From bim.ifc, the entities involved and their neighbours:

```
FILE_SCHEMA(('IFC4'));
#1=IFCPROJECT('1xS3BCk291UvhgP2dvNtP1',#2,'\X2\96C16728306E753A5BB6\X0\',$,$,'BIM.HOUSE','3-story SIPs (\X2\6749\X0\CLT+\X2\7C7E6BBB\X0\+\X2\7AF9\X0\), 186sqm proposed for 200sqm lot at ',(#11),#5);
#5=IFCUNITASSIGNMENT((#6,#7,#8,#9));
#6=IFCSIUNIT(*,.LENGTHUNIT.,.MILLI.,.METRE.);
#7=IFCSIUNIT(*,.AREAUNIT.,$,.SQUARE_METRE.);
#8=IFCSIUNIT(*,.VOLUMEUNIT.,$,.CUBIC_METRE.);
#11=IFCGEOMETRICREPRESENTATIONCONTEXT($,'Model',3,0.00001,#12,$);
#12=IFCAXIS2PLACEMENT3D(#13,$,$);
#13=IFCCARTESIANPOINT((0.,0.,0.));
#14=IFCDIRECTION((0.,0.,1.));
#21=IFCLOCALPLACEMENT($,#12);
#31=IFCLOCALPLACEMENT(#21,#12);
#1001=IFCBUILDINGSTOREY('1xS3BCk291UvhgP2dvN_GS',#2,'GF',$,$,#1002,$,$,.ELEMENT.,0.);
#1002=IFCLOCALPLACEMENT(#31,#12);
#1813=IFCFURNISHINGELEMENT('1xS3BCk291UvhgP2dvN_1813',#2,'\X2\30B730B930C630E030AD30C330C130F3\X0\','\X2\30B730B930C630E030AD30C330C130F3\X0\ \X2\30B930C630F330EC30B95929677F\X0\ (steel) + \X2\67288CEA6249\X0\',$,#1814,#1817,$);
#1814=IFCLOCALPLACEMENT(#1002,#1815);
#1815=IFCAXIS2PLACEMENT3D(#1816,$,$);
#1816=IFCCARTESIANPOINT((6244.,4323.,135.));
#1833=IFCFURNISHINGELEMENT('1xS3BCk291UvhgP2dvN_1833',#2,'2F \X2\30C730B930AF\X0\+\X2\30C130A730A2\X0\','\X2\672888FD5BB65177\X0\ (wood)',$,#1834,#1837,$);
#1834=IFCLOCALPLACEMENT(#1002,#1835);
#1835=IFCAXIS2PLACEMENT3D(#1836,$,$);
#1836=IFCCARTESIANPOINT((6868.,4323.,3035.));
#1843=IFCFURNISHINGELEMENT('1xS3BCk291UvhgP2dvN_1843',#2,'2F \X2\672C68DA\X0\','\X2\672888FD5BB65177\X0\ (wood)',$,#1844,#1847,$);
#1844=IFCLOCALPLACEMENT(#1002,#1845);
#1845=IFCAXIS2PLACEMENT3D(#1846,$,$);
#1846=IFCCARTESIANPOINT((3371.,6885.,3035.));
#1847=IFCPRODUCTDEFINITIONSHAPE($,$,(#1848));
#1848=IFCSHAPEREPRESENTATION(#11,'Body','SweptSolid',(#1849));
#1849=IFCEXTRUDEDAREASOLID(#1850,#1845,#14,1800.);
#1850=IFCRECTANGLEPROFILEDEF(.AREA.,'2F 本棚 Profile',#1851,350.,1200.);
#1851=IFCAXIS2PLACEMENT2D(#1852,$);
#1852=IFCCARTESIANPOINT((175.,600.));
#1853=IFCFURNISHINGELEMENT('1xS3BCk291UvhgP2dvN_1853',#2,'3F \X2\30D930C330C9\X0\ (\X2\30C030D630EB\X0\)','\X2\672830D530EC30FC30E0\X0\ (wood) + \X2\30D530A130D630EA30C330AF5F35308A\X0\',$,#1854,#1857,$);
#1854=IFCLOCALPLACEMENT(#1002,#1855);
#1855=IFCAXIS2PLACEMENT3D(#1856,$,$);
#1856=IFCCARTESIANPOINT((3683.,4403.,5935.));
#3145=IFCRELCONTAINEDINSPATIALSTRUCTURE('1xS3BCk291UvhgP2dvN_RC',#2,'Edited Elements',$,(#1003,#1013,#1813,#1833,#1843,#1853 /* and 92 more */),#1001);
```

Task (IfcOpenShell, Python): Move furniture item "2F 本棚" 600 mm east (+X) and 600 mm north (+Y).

```python
import ifcopenshell
import ifcopenshell.api.geometry
import ifcopenshell.util.placement
import ifcopenshell.util.unit

model = ifcopenshell.open("bim.ifc")
unit_scale = ifcopenshell.util.unit.calculate_unit_scale(model)

item = model.by_id(1843)
matrix = ifcopenshell.util.placement.get_local_placement(item.ObjectPlacement)
matrix[0, 3] += 0.6 / unit_scale
matrix[1, 3] += 0.6 / unit_scale
ifcopenshell.api.geometry.edit_object_placement(model, product=item, matrix=matrix, is_si=False)

print(ifcopenshell.util.placement.get_local_placement(item.ObjectPlacement).round(3) + 0.0)

model.write("bim_v2.ifc")
```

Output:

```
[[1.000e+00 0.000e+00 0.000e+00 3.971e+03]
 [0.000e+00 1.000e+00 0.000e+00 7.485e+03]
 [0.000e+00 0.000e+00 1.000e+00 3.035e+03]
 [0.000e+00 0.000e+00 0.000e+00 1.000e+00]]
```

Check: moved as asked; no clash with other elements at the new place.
